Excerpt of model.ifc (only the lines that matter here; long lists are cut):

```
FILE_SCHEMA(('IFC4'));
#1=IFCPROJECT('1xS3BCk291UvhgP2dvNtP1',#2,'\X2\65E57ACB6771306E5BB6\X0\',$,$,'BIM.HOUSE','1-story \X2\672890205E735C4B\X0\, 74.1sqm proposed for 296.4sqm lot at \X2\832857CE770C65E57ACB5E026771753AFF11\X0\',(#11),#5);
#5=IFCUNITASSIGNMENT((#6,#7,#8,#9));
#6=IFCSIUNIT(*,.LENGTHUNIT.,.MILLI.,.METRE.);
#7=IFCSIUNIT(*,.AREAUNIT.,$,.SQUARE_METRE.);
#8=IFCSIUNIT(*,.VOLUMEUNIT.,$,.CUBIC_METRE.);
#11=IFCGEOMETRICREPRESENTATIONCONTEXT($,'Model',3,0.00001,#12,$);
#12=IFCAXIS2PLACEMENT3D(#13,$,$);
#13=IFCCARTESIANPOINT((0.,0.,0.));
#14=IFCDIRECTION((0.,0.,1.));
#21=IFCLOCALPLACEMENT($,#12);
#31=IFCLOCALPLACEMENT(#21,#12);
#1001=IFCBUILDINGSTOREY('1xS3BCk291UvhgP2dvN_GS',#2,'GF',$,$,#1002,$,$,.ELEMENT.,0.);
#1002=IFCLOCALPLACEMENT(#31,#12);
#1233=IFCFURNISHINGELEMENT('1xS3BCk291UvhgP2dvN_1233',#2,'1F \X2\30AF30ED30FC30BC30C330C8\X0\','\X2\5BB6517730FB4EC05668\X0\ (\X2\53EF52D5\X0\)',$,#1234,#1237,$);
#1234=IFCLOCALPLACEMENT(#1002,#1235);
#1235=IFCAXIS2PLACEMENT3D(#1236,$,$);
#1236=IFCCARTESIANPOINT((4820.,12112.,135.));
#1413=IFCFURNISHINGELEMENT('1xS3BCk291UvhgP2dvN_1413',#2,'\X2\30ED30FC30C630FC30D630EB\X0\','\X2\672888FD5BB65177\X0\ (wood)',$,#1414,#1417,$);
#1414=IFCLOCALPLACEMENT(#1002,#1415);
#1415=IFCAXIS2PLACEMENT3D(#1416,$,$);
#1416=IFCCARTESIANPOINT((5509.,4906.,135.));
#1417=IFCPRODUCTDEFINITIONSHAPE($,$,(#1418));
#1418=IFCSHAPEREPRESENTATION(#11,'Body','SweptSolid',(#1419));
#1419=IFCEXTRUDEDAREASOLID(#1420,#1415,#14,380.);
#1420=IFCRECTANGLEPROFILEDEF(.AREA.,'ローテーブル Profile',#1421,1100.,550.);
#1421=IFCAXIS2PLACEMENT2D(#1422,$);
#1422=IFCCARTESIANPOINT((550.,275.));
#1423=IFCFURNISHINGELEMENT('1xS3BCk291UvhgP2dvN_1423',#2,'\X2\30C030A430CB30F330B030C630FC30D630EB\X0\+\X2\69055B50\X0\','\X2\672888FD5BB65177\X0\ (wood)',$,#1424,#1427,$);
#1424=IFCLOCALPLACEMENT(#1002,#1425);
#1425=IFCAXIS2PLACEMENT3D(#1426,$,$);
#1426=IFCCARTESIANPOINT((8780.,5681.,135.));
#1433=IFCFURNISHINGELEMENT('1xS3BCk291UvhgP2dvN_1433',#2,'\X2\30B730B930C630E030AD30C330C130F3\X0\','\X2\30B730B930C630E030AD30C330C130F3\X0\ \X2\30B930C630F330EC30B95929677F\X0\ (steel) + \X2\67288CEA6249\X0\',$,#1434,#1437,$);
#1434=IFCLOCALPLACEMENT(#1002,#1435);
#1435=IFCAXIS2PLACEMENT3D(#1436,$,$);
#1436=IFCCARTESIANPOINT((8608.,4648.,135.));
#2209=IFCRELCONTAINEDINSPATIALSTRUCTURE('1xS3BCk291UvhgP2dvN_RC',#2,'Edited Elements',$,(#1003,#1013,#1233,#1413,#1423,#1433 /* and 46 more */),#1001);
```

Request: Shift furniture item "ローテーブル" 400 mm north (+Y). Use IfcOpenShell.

```python
import ifcopenshell
import ifcopenshell.api.geometry
import ifcopenshell.util.placement
import ifcopenshell.util.unit

model = ifcopenshell.open("model.ifc")
unit_scale = ifcopenshell.util.unit.calculate_unit_scale(model)

item = model.by_guid("1xS3BCk291UvhgP2dvN_1413")
matrix = ifcopenshell.util.placement.get_local_placement(item.ObjectPlacement)
matrix[1, 3] += 0.4 / unit_scale
ifcopenshell.api.geometry.edit_object_placement(model, product=item, matrix=matrix, is_si=False)

print(ifcopenshell.util.placement.get_local_placement(item.ObjectPlacement).round(3) + 0.0)

model.write("model-out.ifc")
```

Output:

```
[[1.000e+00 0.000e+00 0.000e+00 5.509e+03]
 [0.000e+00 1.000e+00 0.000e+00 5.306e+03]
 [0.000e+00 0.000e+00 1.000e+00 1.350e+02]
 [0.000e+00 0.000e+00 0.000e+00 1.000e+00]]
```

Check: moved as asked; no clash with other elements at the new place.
